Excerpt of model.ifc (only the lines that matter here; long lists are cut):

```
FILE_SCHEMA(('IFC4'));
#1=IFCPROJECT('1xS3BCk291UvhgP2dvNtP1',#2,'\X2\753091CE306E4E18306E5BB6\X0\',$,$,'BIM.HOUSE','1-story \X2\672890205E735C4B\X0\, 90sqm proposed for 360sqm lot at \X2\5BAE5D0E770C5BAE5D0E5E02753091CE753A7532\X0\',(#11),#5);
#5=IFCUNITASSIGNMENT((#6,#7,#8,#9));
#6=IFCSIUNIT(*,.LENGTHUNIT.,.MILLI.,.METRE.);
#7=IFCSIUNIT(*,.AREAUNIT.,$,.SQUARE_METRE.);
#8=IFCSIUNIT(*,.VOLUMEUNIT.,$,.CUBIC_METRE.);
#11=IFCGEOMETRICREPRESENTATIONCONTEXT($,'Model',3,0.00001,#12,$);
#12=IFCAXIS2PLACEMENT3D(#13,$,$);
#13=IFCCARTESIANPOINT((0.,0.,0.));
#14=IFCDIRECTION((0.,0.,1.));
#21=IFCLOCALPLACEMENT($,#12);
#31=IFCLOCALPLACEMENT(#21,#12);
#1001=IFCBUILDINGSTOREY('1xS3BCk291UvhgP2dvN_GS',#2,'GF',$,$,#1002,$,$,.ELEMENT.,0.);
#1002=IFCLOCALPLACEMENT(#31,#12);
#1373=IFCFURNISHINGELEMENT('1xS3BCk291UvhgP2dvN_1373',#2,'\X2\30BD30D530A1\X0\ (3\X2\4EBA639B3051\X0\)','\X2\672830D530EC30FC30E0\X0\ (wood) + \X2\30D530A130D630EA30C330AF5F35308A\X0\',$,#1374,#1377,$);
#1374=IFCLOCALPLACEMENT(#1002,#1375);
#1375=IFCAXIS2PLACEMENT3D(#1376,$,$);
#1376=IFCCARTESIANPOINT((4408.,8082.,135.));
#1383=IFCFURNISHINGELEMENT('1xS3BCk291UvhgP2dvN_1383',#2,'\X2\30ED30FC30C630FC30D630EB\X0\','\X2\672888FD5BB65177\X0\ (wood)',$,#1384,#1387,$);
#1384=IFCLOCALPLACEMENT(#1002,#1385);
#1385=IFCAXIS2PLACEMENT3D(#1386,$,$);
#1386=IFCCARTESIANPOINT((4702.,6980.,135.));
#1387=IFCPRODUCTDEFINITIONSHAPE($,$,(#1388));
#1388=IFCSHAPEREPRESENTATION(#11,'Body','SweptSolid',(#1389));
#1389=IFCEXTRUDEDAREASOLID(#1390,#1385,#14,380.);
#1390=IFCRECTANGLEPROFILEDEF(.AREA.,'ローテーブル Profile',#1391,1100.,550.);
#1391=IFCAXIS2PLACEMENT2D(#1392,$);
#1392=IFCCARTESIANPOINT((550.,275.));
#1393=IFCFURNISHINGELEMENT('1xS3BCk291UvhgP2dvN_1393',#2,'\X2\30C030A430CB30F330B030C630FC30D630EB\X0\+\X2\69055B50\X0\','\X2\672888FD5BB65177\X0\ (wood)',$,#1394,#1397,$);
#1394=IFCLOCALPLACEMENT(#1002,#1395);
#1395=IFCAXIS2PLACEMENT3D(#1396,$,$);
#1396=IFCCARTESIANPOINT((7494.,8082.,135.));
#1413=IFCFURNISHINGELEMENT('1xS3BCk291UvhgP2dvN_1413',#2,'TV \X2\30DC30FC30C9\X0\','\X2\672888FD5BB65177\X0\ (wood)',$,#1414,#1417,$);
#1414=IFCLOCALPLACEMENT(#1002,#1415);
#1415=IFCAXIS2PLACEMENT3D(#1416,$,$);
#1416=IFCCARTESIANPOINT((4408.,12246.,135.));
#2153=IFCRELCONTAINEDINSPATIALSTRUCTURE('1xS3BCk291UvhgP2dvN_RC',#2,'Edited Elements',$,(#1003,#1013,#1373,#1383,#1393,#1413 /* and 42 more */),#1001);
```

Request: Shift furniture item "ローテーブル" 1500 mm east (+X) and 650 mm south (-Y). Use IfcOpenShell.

```python
import ifcopenshell
import ifcopenshell.api.geometry
import ifcopenshell.util.placement

model = ifcopenshell.open("model.ifc")

item = model.by_guid("1xS3BCk291UvhgP2dvN_1383")
matrix = ifcopenshell.util.placement.get_local_placement(item.ObjectPlacement)
matrix[0, 3] += 1500.0
matrix[1, 3] -= 650.0
ifcopenshell.api.geometry.edit_object_placement(model, product=item, matrix=matrix, is_si=False)

print(ifcopenshell.util.placement.get_local_placement(item.ObjectPlacement).round(3) + 0.0)

model.write("model-out.ifc")
```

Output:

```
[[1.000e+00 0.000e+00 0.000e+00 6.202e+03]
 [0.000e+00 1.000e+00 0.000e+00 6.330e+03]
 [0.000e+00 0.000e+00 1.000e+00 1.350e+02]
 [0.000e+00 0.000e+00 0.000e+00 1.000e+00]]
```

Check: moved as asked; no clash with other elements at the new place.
